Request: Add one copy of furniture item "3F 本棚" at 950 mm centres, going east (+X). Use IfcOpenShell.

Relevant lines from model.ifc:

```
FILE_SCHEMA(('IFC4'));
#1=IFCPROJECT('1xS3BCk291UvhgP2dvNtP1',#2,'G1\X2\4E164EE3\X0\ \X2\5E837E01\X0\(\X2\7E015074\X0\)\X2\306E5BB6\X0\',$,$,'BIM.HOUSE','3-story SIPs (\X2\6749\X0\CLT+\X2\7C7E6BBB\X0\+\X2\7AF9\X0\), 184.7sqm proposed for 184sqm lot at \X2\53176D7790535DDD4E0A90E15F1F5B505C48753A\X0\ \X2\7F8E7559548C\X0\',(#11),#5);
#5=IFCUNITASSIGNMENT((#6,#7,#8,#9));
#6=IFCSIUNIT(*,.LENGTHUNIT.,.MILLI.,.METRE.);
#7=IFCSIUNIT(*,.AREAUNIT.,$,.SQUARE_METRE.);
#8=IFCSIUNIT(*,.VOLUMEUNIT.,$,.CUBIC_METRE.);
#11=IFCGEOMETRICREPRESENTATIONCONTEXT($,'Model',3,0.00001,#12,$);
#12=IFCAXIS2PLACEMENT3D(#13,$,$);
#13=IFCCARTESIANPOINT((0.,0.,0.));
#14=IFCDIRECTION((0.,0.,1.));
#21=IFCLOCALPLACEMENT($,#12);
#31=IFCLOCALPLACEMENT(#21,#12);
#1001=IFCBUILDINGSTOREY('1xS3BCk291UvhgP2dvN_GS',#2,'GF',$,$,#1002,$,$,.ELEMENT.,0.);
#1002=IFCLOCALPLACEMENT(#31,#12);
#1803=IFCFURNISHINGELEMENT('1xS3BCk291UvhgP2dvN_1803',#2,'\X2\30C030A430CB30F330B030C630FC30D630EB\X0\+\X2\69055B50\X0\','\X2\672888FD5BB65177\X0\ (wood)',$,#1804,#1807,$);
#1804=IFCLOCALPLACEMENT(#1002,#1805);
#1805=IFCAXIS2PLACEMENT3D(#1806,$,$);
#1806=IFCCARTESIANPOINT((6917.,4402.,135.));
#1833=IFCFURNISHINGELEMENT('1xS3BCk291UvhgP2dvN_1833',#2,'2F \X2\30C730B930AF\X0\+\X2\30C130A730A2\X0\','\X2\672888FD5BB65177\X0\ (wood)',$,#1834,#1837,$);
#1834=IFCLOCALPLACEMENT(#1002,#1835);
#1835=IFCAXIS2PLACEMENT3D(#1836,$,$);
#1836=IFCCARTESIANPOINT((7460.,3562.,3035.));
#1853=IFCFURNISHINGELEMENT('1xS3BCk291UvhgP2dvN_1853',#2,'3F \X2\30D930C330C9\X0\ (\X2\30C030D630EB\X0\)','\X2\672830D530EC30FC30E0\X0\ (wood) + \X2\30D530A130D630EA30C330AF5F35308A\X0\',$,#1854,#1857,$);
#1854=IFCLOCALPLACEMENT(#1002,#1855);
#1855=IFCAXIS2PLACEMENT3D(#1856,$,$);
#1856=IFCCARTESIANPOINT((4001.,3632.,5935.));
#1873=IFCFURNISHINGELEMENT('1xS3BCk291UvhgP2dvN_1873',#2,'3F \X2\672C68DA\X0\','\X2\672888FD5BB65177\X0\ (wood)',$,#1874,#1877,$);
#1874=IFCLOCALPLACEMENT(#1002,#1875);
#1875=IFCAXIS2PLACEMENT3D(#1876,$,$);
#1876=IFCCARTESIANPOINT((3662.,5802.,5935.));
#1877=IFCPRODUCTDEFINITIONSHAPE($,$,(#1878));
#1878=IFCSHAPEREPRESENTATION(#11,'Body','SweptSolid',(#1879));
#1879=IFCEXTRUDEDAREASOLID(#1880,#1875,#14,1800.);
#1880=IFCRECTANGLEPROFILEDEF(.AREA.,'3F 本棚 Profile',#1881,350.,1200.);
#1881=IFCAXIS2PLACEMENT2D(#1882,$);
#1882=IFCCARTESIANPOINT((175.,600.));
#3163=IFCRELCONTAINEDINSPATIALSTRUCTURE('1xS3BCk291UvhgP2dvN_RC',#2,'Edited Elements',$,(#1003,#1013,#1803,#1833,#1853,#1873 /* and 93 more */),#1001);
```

```python
import numpy as np
import ifcopenshell
import ifcopenshell.api.geometry
import ifcopenshell.api.root
import ifcopenshell.util.element
import ifcopenshell.util.placement

model = ifcopenshell.open("model.ifc")


def reuse_history(source, copy):
    """copy_class also copies each property set's owner history, people and application; keep the originals."""
    for rel in copy.IsDefinedBy:
        if rel.is_a("IfcRelDefinesByProperties") and (history := rel.RelatingPropertyDefinition.OwnerHistory):
            rel.RelatingPropertyDefinition.OwnerHistory = source.OwnerHistory
            ifcopenshell.util.element.remove_deep2(model, history)


source = model.by_id(1873)
base = ifcopenshell.util.placement.get_local_placement(source.ObjectPlacement)
step = np.array([1.0, 0.0, 0.0]) * 950.0

for i in range(1, 2):
    copy = ifcopenshell.api.root.copy_class(model, product=source)
    copy.Representation = ifcopenshell.util.element.copy_deep(
        model, source.Representation, exclude=["IfcGeometricRepresentationContext", "IfcRepresentationMap"]
    )
    reuse_history(source, copy)
    matrix = base.copy()
    matrix[:3, 3] += i * step
    print("added at", matrix[:3, 3].round(3) + 0.0)
    ifcopenshell.api.geometry.edit_object_placement(model, product=copy, matrix=matrix, is_si=False)

model.write("model-out.ifc")
```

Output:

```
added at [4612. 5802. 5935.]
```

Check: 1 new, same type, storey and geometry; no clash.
